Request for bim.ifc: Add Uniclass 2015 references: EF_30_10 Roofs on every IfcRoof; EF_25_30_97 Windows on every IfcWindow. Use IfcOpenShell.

First a look at what the model holds.

```python
import ifcopenshell

model = ifcopenshell.open("bim.ifc")
print(model.schema)
print("classifications:", [c.Name for c in model.by_type("IfcClassification")])
for ifc_class in ("IfcDoor", "IfcRoof", "IfcStair", "IfcWall", "IfcWindow"):
    print(ifc_class, len(model.by_type(ifc_class)))
```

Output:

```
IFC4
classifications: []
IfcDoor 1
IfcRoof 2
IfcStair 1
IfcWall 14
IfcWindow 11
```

```python
import ifcopenshell
import ifcopenshell.api.classification

model = ifcopenshell.open("bim.ifc")

system = ifcopenshell.api.classification.add_classification(model, classification="Uniclass 2015")

codes = {
    "IfcRoof": ("EF_30_10", "Roofs"),
    "IfcWindow": ("EF_25_30_97", "Windows"),
}
for ifc_class, (code, name) in codes.items():
    products = model.by_type(ifc_class)
    ifcopenshell.api.classification.add_reference(
        model, products=products, classification=system, identification=code, name=name
    )
    print(code, len(products))

model.write("bim-out.ifc")
```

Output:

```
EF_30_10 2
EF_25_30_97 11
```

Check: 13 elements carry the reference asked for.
